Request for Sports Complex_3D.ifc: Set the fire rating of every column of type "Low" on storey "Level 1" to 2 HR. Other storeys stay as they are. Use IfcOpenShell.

First a look at what the model holds.

```python
import ifcopenshell
import ifcopenshell.util.element

model = ifcopenshell.open("Sports Complex_3D.ifc")
print(model.schema)
storey = next(s for s in model.by_type("IfcBuildingStorey") if s.Name == "Level 1")
columns = [e for e in ifcopenshell.util.element.get_decomposition(storey) if e.is_a("IfcColumn")]
seen = {}
for e in columns:
    element_type = ifcopenshell.util.element.get_type(e)
    key = (element_type.Name if element_type != e and element_type else None, ifcopenshell.util.element.get_pset(e, "Pset_ColumnCommon", "FireRating"))
    seen[key] = seen.get(key, 0) + 1
for (name, value), count in sorted(seen.items(), key=str):
    print(count, "x", name, "|", value)
```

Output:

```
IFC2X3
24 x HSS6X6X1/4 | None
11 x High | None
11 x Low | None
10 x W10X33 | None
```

```python
import ifcopenshell
import ifcopenshell.api.pset
import ifcopenshell.util.element

model = ifcopenshell.open("Sports Complex_3D.ifc")

storey = next(s for s in model.by_type("IfcBuildingStorey") if s.Name == "Level 1")
columns = [e for e in ifcopenshell.util.element.get_decomposition(storey) if e.is_a("IfcColumn")]

count = 0
for e in columns:
    element_type = ifcopenshell.util.element.get_type(e)
    if element_type in (None, e) or element_type.Name != "Low":
        continue
    # add_pset returns the element's existing set when there is one.
    pset = ifcopenshell.api.pset.add_pset(model, product=e, name="Pset_ColumnCommon")
    ifcopenshell.api.pset.edit_pset(model, pset=pset, properties={"FireRating": "2 HR"})
    count += 1

print(count, "columns updated")

model.write("Sports Complex_3D_edited.ifc")
```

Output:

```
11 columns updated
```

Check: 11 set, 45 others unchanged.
